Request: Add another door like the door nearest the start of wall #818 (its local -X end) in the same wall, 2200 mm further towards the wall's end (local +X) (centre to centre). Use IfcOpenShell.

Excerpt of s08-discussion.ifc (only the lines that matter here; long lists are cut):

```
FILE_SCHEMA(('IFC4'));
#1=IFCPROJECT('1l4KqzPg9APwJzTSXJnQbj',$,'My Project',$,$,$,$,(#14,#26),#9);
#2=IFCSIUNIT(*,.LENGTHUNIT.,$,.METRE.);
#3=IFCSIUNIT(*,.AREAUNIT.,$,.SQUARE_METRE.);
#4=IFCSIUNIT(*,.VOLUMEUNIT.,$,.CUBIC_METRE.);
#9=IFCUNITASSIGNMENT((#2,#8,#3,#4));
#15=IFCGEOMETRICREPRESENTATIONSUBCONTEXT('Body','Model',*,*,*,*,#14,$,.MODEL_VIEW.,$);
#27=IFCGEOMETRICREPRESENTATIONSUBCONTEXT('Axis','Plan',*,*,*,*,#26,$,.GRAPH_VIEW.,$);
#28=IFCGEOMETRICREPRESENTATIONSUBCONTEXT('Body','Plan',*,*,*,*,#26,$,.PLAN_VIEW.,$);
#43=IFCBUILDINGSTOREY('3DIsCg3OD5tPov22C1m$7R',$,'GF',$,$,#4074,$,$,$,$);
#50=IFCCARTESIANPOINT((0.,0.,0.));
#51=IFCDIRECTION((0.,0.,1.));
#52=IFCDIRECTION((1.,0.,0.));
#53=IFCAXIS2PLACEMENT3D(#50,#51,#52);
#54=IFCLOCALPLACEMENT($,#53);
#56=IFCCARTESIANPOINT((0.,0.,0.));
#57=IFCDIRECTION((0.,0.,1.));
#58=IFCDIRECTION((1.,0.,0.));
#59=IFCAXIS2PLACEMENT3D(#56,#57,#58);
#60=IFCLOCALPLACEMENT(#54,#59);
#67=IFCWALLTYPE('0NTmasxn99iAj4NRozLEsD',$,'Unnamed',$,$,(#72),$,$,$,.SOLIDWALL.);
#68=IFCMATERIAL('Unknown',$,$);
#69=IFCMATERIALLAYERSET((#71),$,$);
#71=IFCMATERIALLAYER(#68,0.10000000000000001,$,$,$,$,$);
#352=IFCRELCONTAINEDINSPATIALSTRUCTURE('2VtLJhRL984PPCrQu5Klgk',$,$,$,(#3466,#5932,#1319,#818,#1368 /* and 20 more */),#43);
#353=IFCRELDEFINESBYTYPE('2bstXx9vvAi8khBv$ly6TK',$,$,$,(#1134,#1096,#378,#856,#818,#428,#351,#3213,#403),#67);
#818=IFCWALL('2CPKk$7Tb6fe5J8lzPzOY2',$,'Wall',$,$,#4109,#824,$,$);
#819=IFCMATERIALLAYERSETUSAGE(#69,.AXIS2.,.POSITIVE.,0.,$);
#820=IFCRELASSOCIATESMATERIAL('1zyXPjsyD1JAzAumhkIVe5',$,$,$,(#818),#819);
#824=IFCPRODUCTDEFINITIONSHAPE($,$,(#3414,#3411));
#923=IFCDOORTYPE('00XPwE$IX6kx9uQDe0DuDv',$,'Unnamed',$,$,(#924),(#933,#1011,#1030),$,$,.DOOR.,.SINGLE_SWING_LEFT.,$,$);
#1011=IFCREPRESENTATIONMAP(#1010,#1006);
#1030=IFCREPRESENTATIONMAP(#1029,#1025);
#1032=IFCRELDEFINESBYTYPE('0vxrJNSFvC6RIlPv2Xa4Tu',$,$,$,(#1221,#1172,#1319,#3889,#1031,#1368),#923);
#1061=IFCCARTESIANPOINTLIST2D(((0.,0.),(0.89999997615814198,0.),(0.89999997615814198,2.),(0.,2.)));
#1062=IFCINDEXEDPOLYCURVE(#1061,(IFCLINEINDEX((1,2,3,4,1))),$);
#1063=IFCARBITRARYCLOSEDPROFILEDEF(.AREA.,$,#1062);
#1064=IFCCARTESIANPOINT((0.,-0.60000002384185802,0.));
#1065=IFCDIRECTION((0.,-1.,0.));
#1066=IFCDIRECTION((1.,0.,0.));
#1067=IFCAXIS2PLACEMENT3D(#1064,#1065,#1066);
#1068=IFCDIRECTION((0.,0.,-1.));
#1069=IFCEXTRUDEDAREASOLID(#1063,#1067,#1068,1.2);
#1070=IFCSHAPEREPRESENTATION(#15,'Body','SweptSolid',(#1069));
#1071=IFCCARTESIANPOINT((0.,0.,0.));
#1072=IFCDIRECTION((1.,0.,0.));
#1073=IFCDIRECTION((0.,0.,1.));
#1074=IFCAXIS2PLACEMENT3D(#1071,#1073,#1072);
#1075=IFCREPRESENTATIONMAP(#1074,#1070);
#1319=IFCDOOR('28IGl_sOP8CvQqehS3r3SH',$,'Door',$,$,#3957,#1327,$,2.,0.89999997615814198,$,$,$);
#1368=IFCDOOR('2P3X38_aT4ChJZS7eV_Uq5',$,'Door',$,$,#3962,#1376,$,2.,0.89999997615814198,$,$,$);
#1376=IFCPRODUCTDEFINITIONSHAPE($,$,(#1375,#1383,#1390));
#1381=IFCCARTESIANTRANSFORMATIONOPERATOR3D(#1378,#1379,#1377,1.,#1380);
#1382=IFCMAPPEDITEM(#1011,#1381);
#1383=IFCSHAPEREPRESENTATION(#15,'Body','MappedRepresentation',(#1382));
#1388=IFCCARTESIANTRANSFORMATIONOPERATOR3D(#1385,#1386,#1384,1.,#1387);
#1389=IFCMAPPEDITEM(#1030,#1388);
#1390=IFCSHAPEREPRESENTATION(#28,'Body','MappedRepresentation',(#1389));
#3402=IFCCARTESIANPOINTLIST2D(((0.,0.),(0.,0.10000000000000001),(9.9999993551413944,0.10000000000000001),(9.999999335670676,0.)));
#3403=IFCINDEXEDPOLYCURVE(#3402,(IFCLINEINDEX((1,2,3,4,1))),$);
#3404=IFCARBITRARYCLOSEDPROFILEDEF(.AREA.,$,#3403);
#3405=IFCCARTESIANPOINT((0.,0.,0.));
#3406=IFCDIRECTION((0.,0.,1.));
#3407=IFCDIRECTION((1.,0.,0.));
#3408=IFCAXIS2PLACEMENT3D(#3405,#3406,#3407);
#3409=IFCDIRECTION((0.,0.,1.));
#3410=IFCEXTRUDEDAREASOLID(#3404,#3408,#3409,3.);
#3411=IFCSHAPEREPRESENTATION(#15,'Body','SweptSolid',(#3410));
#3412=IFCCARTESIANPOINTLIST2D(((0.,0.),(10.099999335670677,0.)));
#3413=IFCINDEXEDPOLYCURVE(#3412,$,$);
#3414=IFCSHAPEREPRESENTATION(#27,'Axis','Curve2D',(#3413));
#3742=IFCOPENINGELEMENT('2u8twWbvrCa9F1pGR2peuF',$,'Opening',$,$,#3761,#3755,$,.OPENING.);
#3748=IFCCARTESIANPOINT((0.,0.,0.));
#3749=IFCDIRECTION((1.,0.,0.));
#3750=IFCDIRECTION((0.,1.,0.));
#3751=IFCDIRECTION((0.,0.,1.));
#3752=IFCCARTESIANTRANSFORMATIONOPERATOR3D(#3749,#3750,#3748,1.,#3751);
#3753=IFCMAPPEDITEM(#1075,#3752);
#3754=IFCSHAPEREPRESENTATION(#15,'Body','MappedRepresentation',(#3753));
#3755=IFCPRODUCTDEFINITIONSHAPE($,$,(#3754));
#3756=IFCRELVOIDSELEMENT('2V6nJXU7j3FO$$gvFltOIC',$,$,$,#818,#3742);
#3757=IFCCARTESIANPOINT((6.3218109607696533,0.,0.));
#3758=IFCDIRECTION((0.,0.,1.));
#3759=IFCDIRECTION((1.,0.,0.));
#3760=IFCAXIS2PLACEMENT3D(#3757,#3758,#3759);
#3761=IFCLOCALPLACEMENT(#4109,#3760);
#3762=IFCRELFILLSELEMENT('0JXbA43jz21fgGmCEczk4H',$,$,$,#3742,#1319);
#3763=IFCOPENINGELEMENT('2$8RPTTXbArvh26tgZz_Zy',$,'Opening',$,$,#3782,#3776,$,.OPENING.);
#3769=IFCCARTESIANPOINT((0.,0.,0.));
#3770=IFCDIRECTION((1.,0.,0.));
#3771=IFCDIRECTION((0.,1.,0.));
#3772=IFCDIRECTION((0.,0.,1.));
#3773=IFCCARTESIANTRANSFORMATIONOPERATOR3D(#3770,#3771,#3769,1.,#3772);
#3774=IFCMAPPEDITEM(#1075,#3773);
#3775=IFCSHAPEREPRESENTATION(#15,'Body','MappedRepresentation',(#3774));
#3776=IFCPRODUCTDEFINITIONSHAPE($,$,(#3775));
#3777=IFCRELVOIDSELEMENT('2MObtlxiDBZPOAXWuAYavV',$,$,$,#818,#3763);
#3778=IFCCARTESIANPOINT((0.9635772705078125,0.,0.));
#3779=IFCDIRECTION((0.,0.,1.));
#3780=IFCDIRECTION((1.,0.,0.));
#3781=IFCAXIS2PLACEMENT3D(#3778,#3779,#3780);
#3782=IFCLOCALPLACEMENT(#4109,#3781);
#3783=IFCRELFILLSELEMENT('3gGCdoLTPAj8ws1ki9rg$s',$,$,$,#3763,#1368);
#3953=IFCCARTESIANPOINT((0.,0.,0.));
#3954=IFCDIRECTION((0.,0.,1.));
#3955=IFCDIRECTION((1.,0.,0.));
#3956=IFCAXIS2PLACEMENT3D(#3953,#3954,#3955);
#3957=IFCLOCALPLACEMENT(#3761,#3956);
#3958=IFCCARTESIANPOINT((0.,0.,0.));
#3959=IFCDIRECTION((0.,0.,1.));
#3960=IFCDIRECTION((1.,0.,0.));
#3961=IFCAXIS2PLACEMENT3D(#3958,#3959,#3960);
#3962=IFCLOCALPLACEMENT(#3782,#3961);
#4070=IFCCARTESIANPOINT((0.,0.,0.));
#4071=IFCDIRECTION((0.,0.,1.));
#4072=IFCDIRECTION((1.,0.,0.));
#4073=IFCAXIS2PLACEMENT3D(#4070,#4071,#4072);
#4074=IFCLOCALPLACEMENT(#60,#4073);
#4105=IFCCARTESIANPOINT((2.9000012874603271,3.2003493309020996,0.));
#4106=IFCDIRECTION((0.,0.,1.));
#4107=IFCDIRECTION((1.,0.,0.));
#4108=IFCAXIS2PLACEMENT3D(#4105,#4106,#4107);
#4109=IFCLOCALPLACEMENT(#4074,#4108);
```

```python
import ifcopenshell
import ifcopenshell.api.feature
import ifcopenshell.api.geometry
import ifcopenshell.api.root
import ifcopenshell.geom
import ifcopenshell.util.element
import ifcopenshell.util.placement
import ifcopenshell.util.shape

model = ifcopenshell.open("s08-discussion.ifc")
settings = ifcopenshell.geom.settings()


def volume(element):
    """Net volume in cubic metres, openings subtracted."""
    shape = ifcopenshell.geom.create_shape(settings, element)
    return ifcopenshell.util.shape.get_volume(shape.geometry)


door = model.by_guid("2P3X38_aT4ChJZS7eV_Uq5")
opening = door.FillsVoids[0].RelatingOpeningElement
wall = opening.VoidsElements[0].RelatingBuildingElement
before = volume(wall)
shift = ifcopenshell.util.placement.get_local_placement(wall.ObjectPlacement)[:3, 0] * 2.2

# copy_class copies the void relationship, type, container and properties, but no geometry.
new_opening = ifcopenshell.api.root.copy_class(model, product=opening)
new_opening.Representation = ifcopenshell.util.element.copy_deep(
    model, opening.Representation, exclude=["IfcGeometricRepresentationContext", "IfcRepresentationMap"]
)
new_door = ifcopenshell.api.root.copy_class(model, product=door)
new_door.Representation = ifcopenshell.util.element.copy_deep(
    model, door.Representation, exclude=["IfcGeometricRepresentationContext", "IfcRepresentationMap"]
)
ifcopenshell.api.feature.add_filling(model, opening=new_opening, element=new_door)

for old, new in ((opening, new_opening), (door, new_door)):
    matrix = ifcopenshell.util.placement.get_local_placement(old.ObjectPlacement)
    matrix[:3, 3] += shift
    ifcopenshell.api.geometry.edit_object_placement(model, product=new, matrix=matrix, is_si=False)

after = volume(wall)

print(f"wall volume {before:.3f} -> {after:.3f} m3")

model.write("s08-discussion_edited.ifc")
```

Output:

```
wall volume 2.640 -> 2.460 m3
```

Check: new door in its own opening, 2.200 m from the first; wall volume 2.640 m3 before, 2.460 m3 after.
